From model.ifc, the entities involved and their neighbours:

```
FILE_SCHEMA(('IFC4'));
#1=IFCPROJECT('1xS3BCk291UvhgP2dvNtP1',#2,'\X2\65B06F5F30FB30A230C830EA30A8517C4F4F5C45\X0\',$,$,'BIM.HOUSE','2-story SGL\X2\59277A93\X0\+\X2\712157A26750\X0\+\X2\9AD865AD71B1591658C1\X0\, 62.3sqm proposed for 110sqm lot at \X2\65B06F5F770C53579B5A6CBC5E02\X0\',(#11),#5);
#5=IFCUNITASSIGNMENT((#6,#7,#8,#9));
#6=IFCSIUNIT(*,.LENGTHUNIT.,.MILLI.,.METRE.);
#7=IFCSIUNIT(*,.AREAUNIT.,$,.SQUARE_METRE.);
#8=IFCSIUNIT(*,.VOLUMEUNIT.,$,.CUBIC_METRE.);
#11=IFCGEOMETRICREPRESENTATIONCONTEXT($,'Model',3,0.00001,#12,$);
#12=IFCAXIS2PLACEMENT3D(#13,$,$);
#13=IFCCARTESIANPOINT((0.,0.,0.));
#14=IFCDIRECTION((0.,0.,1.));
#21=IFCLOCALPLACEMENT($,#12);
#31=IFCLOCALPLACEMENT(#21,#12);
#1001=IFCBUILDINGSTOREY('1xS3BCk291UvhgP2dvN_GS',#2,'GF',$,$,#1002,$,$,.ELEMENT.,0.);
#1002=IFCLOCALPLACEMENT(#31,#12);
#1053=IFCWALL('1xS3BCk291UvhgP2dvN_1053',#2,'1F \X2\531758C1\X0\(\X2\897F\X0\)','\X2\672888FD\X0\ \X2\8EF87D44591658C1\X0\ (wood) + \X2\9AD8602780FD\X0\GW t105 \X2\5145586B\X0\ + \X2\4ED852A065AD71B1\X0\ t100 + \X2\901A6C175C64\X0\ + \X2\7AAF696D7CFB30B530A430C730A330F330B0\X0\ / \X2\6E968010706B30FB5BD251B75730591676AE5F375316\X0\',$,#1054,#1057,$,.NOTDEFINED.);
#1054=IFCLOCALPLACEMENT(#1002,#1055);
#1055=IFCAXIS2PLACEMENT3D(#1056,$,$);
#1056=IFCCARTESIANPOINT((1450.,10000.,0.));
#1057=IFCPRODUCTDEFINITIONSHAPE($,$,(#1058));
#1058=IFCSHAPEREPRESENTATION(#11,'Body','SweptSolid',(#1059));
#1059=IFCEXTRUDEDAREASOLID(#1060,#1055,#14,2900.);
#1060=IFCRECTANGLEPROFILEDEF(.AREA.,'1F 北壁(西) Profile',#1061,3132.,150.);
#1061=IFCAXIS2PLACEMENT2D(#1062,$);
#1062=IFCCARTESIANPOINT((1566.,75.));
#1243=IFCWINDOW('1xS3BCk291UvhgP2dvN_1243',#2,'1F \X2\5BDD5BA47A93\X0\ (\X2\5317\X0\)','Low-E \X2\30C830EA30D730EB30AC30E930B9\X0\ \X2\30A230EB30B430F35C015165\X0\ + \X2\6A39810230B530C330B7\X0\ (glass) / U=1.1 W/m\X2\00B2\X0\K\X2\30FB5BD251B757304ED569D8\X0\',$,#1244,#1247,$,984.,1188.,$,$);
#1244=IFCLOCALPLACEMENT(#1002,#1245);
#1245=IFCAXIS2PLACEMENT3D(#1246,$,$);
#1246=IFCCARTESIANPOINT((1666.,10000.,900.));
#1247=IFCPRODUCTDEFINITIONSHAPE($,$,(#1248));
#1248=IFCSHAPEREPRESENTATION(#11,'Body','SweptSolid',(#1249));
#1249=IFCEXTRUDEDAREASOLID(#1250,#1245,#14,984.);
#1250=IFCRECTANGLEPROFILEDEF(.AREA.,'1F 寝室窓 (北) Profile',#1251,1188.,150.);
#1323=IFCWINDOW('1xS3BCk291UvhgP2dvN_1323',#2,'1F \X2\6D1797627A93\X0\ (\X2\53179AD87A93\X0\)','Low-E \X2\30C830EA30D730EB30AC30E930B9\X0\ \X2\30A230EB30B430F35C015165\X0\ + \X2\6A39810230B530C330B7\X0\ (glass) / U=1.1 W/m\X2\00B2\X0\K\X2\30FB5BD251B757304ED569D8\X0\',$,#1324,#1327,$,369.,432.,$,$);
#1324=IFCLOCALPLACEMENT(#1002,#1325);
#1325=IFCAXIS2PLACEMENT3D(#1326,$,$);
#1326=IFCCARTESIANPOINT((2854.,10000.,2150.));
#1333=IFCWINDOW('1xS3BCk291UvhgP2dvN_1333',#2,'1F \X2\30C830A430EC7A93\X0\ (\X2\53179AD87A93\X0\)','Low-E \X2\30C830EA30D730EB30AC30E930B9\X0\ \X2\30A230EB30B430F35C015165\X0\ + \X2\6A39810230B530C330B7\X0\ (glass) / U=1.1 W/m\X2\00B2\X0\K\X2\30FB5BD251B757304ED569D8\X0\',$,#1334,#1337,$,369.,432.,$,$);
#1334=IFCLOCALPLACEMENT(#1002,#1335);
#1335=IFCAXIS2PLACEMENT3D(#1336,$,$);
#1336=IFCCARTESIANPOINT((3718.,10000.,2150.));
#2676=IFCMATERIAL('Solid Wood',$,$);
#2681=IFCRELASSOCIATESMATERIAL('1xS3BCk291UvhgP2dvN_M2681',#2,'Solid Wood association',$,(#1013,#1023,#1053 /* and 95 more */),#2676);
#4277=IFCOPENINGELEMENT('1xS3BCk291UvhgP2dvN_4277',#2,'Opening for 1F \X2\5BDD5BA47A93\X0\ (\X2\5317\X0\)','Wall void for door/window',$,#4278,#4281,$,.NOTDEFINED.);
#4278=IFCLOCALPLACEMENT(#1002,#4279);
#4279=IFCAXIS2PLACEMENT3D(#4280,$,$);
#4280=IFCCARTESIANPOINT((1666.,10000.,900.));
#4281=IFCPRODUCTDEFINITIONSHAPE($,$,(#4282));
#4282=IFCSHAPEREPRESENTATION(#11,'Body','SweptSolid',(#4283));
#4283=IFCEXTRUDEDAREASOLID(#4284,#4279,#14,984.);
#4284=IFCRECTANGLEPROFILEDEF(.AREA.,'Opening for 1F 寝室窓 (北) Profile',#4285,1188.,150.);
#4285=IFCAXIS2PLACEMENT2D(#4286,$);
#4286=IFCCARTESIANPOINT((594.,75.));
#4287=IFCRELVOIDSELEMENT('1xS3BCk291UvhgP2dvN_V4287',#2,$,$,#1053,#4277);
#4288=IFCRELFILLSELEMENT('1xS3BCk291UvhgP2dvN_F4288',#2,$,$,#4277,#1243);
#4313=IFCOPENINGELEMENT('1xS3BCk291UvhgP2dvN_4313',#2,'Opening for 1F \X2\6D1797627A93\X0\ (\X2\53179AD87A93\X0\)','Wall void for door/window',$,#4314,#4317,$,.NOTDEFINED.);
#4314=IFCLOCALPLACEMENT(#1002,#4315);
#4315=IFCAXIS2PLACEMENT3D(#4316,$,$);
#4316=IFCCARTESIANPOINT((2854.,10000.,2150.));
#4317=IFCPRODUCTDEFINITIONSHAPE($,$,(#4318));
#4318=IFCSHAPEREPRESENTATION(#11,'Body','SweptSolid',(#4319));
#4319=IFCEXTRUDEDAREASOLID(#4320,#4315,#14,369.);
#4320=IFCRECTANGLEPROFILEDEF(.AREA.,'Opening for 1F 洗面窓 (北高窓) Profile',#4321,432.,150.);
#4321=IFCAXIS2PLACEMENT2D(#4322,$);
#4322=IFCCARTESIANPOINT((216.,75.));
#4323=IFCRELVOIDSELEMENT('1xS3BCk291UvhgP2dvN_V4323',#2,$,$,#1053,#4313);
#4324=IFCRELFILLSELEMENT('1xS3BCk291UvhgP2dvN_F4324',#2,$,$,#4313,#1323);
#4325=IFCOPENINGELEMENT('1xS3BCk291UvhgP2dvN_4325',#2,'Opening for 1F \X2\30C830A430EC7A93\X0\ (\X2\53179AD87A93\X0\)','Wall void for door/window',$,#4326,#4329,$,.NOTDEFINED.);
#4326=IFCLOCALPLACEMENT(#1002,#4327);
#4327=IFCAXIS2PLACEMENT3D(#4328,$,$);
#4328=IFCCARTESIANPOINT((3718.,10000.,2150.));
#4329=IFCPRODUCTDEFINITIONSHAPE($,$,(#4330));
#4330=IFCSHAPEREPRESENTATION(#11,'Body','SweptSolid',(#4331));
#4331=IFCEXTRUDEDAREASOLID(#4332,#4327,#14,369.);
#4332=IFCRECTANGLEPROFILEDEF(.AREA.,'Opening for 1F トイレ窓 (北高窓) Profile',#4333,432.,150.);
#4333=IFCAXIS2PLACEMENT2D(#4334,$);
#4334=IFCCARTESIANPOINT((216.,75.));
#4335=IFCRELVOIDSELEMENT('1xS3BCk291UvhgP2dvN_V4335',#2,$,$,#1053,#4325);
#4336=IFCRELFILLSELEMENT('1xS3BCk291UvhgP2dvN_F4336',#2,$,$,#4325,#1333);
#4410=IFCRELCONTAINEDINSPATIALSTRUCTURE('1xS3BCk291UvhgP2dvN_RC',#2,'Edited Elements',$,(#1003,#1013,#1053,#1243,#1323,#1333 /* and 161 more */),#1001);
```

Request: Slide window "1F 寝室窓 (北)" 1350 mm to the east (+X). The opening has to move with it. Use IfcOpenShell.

```python
import ifcopenshell
import ifcopenshell.api.geometry
import ifcopenshell.util.placement
import ifcopenshell.util.unit

model = ifcopenshell.open("model.ifc")
unit_scale = ifcopenshell.util.unit.calculate_unit_scale(model)

window = model.by_guid("1xS3BCk291UvhgP2dvN_1243")
opening = window.FillsVoids[0].RelatingOpeningElement
wall = opening.VoidsElements[0].RelatingBuildingElement

wall_matrix = ifcopenshell.util.placement.get_local_placement(wall.ObjectPlacement)
shift = wall_matrix[:3, 0] * 1.35 / unit_scale
before = ifcopenshell.util.placement.get_local_placement(window.ObjectPlacement)[:3, 3].copy()

# The window is not placed relative to its opening, so move both.
for product in (opening, window):
    matrix = ifcopenshell.util.placement.get_local_placement(product.ObjectPlacement)
    matrix[:3, 3] += shift
    ifcopenshell.api.geometry.edit_object_placement(model, product=product, matrix=matrix, is_si=False)

after = ifcopenshell.util.placement.get_local_placement(window.ObjectPlacement)[:3, 3]
print("window moved by", (after - before).round(3) + 0.0)

model.write("model_v2.ifc")
```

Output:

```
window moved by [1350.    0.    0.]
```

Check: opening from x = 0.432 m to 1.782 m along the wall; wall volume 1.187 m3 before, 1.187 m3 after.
